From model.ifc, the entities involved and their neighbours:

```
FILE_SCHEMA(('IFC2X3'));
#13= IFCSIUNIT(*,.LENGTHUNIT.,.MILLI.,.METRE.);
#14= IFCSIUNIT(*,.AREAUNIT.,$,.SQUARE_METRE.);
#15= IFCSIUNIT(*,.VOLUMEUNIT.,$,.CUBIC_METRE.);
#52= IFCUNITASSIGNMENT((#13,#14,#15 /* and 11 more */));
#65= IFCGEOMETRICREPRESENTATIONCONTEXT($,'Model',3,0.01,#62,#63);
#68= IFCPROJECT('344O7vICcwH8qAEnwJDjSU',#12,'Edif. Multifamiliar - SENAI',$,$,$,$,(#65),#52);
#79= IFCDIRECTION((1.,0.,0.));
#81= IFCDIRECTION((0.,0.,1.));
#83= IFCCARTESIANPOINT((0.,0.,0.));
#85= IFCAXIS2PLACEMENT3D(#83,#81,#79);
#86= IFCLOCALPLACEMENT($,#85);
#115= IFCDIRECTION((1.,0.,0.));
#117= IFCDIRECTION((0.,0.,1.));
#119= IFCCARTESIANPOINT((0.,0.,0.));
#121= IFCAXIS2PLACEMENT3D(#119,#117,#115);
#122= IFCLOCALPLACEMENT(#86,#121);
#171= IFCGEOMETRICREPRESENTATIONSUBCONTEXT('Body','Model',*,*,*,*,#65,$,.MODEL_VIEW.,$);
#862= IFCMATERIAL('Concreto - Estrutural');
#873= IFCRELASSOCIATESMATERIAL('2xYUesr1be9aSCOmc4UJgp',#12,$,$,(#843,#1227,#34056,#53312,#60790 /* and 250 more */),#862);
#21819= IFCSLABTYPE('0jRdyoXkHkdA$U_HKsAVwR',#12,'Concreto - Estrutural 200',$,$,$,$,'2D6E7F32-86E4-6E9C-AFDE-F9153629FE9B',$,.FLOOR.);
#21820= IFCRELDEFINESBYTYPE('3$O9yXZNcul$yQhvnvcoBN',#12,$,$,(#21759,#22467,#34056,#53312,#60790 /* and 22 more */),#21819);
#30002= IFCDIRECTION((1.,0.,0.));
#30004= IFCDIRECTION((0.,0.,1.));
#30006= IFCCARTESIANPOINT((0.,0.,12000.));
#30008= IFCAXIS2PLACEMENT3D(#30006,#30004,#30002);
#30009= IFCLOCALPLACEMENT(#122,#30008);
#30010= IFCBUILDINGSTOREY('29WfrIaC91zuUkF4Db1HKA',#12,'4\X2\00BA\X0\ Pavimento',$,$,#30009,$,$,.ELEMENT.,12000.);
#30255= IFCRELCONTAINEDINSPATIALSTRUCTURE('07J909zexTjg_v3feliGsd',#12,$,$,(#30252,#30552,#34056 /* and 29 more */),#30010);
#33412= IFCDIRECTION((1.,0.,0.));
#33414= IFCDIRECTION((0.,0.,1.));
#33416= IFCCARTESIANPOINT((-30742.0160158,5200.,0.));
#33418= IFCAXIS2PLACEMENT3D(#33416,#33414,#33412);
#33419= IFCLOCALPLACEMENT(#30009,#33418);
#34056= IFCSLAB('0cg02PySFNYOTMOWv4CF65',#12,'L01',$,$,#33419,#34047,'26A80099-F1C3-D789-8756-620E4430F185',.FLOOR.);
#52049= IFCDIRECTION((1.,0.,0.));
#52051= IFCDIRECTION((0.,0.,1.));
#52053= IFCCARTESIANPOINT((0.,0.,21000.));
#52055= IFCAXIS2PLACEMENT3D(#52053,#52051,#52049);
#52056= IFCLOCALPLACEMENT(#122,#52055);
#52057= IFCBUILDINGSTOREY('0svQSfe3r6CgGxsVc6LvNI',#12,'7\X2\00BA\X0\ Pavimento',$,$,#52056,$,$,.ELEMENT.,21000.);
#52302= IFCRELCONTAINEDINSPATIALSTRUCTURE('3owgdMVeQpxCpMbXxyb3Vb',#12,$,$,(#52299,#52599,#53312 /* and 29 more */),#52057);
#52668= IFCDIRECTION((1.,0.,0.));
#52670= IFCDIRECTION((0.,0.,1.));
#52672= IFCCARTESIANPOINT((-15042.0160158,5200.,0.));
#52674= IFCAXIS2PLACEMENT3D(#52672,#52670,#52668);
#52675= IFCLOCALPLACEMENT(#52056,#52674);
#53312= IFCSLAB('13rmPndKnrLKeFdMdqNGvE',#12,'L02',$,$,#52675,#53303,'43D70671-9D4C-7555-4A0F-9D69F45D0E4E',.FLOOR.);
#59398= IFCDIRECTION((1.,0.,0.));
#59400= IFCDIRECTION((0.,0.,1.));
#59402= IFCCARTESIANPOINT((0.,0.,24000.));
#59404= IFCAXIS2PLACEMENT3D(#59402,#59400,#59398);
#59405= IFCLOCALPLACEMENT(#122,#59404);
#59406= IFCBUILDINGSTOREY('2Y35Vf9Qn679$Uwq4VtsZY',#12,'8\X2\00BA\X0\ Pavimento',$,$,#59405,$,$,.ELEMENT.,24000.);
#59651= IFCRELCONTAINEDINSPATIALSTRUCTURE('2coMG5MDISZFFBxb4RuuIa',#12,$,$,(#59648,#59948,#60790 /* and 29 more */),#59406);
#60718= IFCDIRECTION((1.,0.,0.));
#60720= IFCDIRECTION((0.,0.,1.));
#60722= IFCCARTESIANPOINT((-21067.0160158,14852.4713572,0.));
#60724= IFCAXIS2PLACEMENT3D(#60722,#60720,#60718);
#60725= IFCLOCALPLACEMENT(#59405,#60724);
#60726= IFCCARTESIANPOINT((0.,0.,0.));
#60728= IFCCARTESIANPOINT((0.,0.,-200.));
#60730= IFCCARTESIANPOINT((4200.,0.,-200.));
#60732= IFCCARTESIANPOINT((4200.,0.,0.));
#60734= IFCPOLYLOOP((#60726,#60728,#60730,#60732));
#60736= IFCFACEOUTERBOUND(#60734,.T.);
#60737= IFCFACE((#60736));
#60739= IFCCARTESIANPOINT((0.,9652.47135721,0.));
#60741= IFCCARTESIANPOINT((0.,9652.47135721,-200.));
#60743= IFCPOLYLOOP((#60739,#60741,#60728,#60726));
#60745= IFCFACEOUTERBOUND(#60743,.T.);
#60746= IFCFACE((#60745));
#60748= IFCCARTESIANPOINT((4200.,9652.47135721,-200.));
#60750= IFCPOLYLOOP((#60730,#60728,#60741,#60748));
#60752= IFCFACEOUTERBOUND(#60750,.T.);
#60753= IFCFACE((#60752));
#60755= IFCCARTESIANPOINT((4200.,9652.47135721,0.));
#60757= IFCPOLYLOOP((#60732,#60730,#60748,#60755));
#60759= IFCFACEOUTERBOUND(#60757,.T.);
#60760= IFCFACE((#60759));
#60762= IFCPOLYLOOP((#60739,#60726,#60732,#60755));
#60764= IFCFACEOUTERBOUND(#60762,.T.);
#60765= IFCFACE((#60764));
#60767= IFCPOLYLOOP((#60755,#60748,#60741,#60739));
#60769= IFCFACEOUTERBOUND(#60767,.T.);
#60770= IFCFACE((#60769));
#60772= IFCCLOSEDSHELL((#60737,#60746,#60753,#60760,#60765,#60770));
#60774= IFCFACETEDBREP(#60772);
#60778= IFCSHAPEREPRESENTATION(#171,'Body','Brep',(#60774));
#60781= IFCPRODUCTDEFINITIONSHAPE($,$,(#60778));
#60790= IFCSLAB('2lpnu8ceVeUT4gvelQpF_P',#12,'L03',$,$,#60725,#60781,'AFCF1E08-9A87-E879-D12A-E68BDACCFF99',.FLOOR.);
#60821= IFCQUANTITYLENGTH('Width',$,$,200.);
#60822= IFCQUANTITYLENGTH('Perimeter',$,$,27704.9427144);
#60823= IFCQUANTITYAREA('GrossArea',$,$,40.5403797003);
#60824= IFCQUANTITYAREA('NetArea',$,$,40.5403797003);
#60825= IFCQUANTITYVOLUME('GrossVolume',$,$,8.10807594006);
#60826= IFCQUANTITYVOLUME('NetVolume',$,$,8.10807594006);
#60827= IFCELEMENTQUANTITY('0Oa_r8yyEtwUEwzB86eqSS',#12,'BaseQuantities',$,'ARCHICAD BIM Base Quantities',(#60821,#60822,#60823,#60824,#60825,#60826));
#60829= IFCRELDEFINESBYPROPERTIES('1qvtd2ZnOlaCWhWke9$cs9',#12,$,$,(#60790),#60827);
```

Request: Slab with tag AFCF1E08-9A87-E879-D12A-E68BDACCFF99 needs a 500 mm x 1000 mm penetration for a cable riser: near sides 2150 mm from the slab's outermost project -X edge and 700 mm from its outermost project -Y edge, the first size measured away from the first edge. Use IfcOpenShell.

```python
import numpy as np
import ifcopenshell
import ifcopenshell.api.feature
import ifcopenshell.api.geometry
import ifcopenshell.api.pset
import ifcopenshell.api.root
import ifcopenshell.geom
import ifcopenshell.util.element
import ifcopenshell.util.placement
import ifcopenshell.util.representation
import ifcopenshell.util.shape
import ifcopenshell.util.unit

model = ifcopenshell.open("model.ifc")
unit_scale = ifcopenshell.util.unit.calculate_unit_scale(model)
area_scale = ifcopenshell.util.unit.calculate_unit_scale(model, "AREAUNIT")
volume_scale = ifcopenshell.util.unit.calculate_unit_scale(model, "VOLUMEUNIT")
settings = ifcopenshell.geom.settings()


def volume(element):
    """Net volume in cubic metres, openings subtracted."""
    shape = ifcopenshell.geom.create_shape(settings, element)
    return ifcopenshell.util.shape.get_volume(shape.geometry)


slab = model.by_guid("2lpnu8ceVeUT4gvelQpF_P")
before = volume(slab)

# Extent in the slab's own axes, in metres. The edges named are its -X and -Y sides.
slab_shape = ifcopenshell.geom.create_shape(settings, slab)
vertices = ifcopenshell.util.shape.get_vertices(slab_shape.geometry)
x_min, y_min, bottom = vertices.min(axis=0)
top = vertices[:, 2].max()

opening = ifcopenshell.api.root.create_entity(model, ifc_class="IfcOpeningElement", name="Cable riser opening")
context = ifcopenshell.util.representation.get_context(model, "Model", "Body", "MODEL_VIEW")
width, depth = 0.5, 1
outline = [(0.0, 0.0), (width, 0.0), (width, depth), (0.0, depth), (0.0, 0.0)]
# Overshoot both faces by 50 mm so the cut is clean.
shape = ifcopenshell.api.geometry.add_slab_representation(
    model, context=context, depth=top - bottom + 0.1, polyline=outline
)
ifcopenshell.api.geometry.assign_representation(model, product=opening, representation=shape)

matrix = ifcopenshell.util.placement.get_local_placement(slab.ObjectPlacement)
matrix[:, 3] = matrix @ np.append(np.array([x_min + 2.15, y_min + 0.7, bottom - 0.05]) / unit_scale, 1.0)
ifcopenshell.api.geometry.edit_object_placement(model, product=opening, matrix=matrix, is_si=False)
ifcopenshell.api.feature.add_feature(model, feature=opening, element=slab)

after = volume(slab)

# Update the slab's stored quantities.
qto = model.by_id(ifcopenshell.util.element.get_pset(slab, "BaseQuantities", should_inherit=False)["id"])
ifcopenshell.api.pset.edit_qto(model, qto=qto, properties={
    "NetArea": after / (top - bottom) / area_scale,
    "NetVolume": after / volume_scale,
})

print(f"slab volume {before:.3f} -> {after:.3f} m3")

model.write("model_v2.ifc")
```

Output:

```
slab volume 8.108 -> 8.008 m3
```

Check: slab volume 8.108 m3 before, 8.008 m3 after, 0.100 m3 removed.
